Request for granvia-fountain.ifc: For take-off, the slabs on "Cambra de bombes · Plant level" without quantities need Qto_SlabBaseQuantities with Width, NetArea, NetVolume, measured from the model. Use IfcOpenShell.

First a look at what the model holds.

```python
import ifcopenshell
import ifcopenshell.util.element
import ifcopenshell.util.unit

model = ifcopenshell.open("granvia-fountain.ifc")
print(model.schema)
for unit_type in ("LENGTHUNIT", "AREAUNIT", "VOLUMEUNIT"):
    print(unit_type, ifcopenshell.util.unit.calculate_unit_scale(model, unit_type))
storey = next(s for s in model.by_type("IfcBuildingStorey") if s.Name == "Cambra de bombes · Plant level")
slabs = [e for e in ifcopenshell.util.element.get_decomposition(storey) if e.is_a("IfcSlab")]
for e in sorted(slabs, key=lambda e: e.id()):
    print(e.id(), e.is_a(), e.Name, list(ifcopenshell.util.element.get_psets(e, qtos_only=True)), sep=" | ")
```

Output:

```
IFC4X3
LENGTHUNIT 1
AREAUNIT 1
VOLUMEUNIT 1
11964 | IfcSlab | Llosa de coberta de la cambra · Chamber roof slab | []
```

```python
import ifcopenshell
import ifcopenshell.api.pset
import ifcopenshell.geom
import ifcopenshell.util.element
import ifcopenshell.util.shape
import ifcopenshell.util.unit

model = ifcopenshell.open("granvia-fountain.ifc")
unit_scale = ifcopenshell.util.unit.calculate_unit_scale(model)
area_scale = ifcopenshell.util.unit.calculate_unit_scale(model, "AREAUNIT")
volume_scale = ifcopenshell.util.unit.calculate_unit_scale(model, "VOLUMEUNIT")
settings = ifcopenshell.geom.settings()

storey = next(s for s in model.by_type("IfcBuildingStorey") if s.Name == "Cambra de bombes · Plant level")
slabs = [e for e in ifcopenshell.util.element.get_decomposition(storey) if e.is_a("IfcSlab")]

for e in sorted(slabs, key=lambda e: e.id()):
    if ifcopenshell.util.element.get_psets(e, qtos_only=True, should_inherit=False):
        continue
    # Geometry comes back in metres, in the element's own axes.
    shape = ifcopenshell.geom.create_shape(settings, e)
    values = {
        "Width": ifcopenshell.util.shape.get_z(shape.geometry) / unit_scale,
        "NetArea": ifcopenshell.util.shape.get_footprint_area(shape.geometry) / area_scale,
        "NetVolume": ifcopenshell.util.shape.get_volume(shape.geometry) / volume_scale,
    }
    qto = ifcopenshell.api.pset.add_qto(model, product=e, name="Qto_SlabBaseQuantities")
    ifcopenshell.api.pset.edit_qto(model, qto=qto, properties=values)
    print(e.id(), {k: round(v, 3) for k, v in values.items()})

model.write("granvia-fountain_v2.ifc")
```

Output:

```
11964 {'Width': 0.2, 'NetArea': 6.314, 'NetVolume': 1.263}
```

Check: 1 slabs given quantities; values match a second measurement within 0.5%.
